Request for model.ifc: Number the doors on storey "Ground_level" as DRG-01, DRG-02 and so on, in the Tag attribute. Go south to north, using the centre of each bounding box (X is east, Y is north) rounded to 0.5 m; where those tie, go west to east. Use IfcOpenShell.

First a look at what the model holds.

```python
import ifcopenshell
import ifcopenshell.util.element
import ifcopenshell.util.placement

model = ifcopenshell.open("model.ifc")
print(model.schema)
storey = next(s for s in model.by_type("IfcBuildingStorey") if s.Name == "Ground_level")
doors = [e for e in ifcopenshell.util.element.get_decomposition(storey) if e.is_a("IfcDoor")]
for e in sorted(doors, key=lambda e: e.id()):
    origin = ifcopenshell.util.placement.get_local_placement(e.ObjectPlacement)[:3, 3]
    print(e.id(), e.Tag, e.Name, origin.round(2) + 0.0, sep=" | ")
```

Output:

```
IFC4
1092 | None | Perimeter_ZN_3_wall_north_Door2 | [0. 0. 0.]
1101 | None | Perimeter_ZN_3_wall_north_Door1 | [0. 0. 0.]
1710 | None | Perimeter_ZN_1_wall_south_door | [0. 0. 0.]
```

```python
import ifcopenshell
import ifcopenshell.geom
import ifcopenshell.util.element
import ifcopenshell.util.shape

model = ifcopenshell.open("model.ifc")
settings = ifcopenshell.geom.settings()
settings.set("use-world-coords", True)


def centre(element):
    shape = ifcopenshell.geom.create_shape(settings, element)
    return ifcopenshell.util.shape.get_bbox_centroid(shape.geometry)


storey = next(s for s in model.by_type("IfcBuildingStorey") if s.Name == "Ground_level")
doors = [e for e in ifcopenshell.util.element.get_decomposition(storey) if e.is_a("IfcDoor")]

# Insertion points can sit at a corner or the storey origin, so sort by the geometry (in metres).
centres = {e: centre(e) for e in doors}
doors.sort(key=lambda e: (round(centres[e][1] / 0.5), centres[e][0]))

for i, e in enumerate(doors, start=1):
    number = f"DRG-{i:02d}"
    e.Tag = number
    print(e.id(), number)

model.write("model_edited.ifc")
```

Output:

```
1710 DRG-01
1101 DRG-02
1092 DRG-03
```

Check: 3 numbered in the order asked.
